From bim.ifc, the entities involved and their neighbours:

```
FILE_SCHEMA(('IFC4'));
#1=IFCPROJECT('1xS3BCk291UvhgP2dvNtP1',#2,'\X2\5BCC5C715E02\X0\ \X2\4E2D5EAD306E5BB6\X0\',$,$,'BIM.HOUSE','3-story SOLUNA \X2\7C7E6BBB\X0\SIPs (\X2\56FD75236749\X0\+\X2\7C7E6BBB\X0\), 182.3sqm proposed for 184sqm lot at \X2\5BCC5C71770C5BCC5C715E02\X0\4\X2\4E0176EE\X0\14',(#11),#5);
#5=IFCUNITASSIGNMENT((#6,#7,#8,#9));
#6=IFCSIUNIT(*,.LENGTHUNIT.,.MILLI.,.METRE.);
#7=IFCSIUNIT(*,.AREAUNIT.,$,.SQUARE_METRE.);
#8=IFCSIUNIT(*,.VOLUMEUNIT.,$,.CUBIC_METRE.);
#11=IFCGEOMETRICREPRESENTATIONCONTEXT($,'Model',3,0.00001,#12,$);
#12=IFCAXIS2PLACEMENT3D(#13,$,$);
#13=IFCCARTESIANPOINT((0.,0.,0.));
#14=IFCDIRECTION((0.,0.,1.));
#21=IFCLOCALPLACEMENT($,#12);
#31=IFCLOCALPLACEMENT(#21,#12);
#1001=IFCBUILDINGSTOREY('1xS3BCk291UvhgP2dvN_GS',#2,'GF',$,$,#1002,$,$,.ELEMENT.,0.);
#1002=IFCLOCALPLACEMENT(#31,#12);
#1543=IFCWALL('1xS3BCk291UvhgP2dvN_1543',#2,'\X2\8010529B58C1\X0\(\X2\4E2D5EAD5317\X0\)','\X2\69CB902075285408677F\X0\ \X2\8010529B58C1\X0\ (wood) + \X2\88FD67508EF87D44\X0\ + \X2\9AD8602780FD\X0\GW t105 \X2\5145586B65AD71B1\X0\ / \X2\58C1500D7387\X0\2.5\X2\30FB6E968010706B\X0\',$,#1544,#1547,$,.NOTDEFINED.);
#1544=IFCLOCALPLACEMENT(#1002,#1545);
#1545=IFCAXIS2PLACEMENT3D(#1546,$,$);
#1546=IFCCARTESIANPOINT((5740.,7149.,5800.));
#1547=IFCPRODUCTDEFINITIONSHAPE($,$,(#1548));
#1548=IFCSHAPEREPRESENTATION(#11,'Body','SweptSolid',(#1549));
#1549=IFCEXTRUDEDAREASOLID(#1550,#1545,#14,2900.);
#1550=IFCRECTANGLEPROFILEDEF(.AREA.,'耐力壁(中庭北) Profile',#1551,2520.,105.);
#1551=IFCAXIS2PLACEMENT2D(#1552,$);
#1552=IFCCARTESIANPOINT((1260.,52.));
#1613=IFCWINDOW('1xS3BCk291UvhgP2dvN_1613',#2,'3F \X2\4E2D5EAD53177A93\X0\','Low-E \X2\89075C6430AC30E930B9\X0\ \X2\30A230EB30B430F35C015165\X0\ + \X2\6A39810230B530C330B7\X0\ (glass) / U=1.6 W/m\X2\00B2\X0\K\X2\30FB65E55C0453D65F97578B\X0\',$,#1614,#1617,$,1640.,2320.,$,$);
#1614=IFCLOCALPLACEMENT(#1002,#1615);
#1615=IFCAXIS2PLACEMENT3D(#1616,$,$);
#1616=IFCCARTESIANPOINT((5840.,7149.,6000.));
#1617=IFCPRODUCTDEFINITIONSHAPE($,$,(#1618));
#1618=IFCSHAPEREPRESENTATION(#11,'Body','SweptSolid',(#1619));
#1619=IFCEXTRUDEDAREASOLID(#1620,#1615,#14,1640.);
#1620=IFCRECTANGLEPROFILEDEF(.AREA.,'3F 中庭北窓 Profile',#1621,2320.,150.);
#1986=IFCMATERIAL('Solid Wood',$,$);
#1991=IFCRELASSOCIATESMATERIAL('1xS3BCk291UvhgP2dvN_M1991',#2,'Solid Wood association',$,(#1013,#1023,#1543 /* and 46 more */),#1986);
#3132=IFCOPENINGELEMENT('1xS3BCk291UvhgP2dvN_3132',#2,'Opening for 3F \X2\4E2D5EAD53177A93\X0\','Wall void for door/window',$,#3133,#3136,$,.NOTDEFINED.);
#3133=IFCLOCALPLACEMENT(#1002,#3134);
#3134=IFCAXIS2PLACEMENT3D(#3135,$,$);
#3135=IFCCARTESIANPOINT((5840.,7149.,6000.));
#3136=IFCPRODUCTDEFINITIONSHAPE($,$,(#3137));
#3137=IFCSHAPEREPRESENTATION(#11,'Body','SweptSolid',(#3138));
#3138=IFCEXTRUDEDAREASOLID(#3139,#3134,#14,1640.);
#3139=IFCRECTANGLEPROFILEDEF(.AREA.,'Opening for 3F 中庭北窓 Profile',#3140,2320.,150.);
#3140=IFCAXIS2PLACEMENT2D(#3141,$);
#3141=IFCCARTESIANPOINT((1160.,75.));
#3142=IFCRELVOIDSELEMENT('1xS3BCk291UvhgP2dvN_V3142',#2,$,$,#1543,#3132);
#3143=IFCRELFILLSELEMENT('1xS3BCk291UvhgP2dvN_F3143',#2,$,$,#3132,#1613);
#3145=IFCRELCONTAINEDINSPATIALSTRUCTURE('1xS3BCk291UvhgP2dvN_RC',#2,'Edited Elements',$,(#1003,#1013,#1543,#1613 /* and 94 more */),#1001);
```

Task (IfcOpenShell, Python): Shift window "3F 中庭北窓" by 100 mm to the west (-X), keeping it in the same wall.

```python
import ifcopenshell
import ifcopenshell.api.geometry
import ifcopenshell.util.placement

model = ifcopenshell.open("bim.ifc")

window = model.by_id(1613)
opening = window.FillsVoids[0].RelatingOpeningElement
wall = opening.VoidsElements[0].RelatingBuildingElement

wall_matrix = ifcopenshell.util.placement.get_local_placement(wall.ObjectPlacement)
shift = wall_matrix[:3, 0] * -100.0
before = ifcopenshell.util.placement.get_local_placement(window.ObjectPlacement)[:3, 3].copy()

# The window is not placed relative to its opening, so move both.
for product in (opening, window):
    matrix = ifcopenshell.util.placement.get_local_placement(product.ObjectPlacement)
    matrix[:3, 3] += shift
    ifcopenshell.api.geometry.edit_object_placement(model, product=product, matrix=matrix, is_si=False)

after = ifcopenshell.util.placement.get_local_placement(window.ObjectPlacement)[:3, 3]
print("window moved by", (after - before).round(3) + 0.0)

model.write("bim_updated.ifc")
```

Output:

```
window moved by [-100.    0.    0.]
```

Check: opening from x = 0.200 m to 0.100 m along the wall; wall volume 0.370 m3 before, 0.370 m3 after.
